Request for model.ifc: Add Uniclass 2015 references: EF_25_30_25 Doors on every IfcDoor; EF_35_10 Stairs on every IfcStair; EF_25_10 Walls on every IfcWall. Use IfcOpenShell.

First a look at what the model holds.

```python
import ifcopenshell

model = ifcopenshell.open("model.ifc")
print(model.schema)
print("classifications:", [c.Name for c in model.by_type("IfcClassification")])
for ifc_class in ("IfcDoor", "IfcRoof", "IfcStair", "IfcWall", "IfcWindow"):
    print(ifc_class, len(model.by_type(ifc_class)))
```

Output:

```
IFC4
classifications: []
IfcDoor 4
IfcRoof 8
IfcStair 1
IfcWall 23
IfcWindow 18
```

```python
import ifcopenshell
import ifcopenshell.api.classification

model = ifcopenshell.open("model.ifc")

system = ifcopenshell.api.classification.add_classification(model, classification="Uniclass 2015")

codes = {
    "IfcDoor": ("EF_25_30_25", "Doors"),
    "IfcStair": ("EF_35_10", "Stairs"),
    "IfcWall": ("EF_25_10", "Walls"),
}
for ifc_class, (code, name) in codes.items():
    products = model.by_type(ifc_class)
    ifcopenshell.api.classification.add_reference(
        model, products=products, classification=system, identification=code, name=name
    )
    print(code, len(products))

model.write("model_updated.ifc")
```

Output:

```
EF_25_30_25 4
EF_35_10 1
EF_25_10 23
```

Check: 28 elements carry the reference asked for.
